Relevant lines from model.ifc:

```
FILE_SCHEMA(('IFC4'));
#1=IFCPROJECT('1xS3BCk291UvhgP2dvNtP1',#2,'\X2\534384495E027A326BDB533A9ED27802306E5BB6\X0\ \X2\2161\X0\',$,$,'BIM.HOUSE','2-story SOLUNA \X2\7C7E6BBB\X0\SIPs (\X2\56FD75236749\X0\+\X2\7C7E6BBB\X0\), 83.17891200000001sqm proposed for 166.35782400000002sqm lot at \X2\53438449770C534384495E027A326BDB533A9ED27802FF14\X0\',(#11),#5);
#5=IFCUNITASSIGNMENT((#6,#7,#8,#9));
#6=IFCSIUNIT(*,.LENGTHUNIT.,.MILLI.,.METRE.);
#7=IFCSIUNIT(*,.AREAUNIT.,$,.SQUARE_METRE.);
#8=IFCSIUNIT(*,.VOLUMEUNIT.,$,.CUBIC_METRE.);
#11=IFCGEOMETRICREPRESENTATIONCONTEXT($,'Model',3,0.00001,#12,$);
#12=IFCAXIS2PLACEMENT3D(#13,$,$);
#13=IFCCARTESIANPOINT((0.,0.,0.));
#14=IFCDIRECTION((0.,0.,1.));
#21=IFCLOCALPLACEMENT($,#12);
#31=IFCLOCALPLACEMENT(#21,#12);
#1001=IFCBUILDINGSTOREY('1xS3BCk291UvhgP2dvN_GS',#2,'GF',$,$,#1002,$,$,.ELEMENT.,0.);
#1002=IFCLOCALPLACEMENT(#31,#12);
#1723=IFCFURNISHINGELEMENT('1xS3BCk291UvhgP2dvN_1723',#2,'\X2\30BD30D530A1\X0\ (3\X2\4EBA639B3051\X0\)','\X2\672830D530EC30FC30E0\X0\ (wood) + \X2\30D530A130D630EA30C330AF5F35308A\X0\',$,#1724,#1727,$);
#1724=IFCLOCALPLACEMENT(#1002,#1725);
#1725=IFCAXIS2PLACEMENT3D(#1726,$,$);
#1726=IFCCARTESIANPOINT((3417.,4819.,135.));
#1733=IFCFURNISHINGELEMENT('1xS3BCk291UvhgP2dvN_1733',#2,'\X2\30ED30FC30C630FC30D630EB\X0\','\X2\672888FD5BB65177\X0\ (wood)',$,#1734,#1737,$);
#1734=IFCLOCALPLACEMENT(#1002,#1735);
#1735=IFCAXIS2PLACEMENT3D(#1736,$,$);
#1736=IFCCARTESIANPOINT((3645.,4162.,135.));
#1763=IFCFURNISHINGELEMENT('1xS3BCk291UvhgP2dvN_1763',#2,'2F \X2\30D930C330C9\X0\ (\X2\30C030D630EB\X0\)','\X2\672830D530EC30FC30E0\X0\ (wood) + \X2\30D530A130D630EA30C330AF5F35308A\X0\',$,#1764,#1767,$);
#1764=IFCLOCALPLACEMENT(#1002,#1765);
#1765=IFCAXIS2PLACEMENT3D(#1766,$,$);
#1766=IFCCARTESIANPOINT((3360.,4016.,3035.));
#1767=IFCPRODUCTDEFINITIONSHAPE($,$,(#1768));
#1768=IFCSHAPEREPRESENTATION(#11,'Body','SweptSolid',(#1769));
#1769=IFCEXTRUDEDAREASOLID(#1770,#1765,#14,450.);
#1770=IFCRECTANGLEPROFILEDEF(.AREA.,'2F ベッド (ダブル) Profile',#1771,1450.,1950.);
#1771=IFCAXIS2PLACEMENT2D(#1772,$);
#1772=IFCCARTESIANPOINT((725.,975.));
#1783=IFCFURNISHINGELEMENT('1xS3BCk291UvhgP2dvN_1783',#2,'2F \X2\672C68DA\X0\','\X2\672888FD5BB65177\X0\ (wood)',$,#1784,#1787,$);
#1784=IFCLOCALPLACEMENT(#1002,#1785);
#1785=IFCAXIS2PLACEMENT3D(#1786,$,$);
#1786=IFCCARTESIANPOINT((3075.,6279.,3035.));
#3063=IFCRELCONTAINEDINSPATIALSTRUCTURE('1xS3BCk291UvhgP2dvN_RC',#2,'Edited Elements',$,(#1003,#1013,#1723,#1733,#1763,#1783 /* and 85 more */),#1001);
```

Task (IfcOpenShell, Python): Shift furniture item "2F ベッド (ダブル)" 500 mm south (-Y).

```python
import ifcopenshell
import ifcopenshell.api.geometry
import ifcopenshell.util.placement
import ifcopenshell.util.unit

model = ifcopenshell.open("model.ifc")
unit_scale = ifcopenshell.util.unit.calculate_unit_scale(model)

item = model.by_guid("1xS3BCk291UvhgP2dvN_1763")
matrix = ifcopenshell.util.placement.get_local_placement(item.ObjectPlacement)
matrix[1, 3] -= 0.5 / unit_scale
ifcopenshell.api.geometry.edit_object_placement(model, product=item, matrix=matrix, is_si=False)

print(ifcopenshell.util.placement.get_local_placement(item.ObjectPlacement).round(3) + 0.0)

model.write("model_updated.ifc")
```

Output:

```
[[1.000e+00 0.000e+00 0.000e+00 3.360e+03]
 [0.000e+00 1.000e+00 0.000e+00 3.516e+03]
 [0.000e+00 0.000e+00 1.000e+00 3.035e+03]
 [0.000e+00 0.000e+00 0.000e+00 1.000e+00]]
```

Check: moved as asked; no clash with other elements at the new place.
